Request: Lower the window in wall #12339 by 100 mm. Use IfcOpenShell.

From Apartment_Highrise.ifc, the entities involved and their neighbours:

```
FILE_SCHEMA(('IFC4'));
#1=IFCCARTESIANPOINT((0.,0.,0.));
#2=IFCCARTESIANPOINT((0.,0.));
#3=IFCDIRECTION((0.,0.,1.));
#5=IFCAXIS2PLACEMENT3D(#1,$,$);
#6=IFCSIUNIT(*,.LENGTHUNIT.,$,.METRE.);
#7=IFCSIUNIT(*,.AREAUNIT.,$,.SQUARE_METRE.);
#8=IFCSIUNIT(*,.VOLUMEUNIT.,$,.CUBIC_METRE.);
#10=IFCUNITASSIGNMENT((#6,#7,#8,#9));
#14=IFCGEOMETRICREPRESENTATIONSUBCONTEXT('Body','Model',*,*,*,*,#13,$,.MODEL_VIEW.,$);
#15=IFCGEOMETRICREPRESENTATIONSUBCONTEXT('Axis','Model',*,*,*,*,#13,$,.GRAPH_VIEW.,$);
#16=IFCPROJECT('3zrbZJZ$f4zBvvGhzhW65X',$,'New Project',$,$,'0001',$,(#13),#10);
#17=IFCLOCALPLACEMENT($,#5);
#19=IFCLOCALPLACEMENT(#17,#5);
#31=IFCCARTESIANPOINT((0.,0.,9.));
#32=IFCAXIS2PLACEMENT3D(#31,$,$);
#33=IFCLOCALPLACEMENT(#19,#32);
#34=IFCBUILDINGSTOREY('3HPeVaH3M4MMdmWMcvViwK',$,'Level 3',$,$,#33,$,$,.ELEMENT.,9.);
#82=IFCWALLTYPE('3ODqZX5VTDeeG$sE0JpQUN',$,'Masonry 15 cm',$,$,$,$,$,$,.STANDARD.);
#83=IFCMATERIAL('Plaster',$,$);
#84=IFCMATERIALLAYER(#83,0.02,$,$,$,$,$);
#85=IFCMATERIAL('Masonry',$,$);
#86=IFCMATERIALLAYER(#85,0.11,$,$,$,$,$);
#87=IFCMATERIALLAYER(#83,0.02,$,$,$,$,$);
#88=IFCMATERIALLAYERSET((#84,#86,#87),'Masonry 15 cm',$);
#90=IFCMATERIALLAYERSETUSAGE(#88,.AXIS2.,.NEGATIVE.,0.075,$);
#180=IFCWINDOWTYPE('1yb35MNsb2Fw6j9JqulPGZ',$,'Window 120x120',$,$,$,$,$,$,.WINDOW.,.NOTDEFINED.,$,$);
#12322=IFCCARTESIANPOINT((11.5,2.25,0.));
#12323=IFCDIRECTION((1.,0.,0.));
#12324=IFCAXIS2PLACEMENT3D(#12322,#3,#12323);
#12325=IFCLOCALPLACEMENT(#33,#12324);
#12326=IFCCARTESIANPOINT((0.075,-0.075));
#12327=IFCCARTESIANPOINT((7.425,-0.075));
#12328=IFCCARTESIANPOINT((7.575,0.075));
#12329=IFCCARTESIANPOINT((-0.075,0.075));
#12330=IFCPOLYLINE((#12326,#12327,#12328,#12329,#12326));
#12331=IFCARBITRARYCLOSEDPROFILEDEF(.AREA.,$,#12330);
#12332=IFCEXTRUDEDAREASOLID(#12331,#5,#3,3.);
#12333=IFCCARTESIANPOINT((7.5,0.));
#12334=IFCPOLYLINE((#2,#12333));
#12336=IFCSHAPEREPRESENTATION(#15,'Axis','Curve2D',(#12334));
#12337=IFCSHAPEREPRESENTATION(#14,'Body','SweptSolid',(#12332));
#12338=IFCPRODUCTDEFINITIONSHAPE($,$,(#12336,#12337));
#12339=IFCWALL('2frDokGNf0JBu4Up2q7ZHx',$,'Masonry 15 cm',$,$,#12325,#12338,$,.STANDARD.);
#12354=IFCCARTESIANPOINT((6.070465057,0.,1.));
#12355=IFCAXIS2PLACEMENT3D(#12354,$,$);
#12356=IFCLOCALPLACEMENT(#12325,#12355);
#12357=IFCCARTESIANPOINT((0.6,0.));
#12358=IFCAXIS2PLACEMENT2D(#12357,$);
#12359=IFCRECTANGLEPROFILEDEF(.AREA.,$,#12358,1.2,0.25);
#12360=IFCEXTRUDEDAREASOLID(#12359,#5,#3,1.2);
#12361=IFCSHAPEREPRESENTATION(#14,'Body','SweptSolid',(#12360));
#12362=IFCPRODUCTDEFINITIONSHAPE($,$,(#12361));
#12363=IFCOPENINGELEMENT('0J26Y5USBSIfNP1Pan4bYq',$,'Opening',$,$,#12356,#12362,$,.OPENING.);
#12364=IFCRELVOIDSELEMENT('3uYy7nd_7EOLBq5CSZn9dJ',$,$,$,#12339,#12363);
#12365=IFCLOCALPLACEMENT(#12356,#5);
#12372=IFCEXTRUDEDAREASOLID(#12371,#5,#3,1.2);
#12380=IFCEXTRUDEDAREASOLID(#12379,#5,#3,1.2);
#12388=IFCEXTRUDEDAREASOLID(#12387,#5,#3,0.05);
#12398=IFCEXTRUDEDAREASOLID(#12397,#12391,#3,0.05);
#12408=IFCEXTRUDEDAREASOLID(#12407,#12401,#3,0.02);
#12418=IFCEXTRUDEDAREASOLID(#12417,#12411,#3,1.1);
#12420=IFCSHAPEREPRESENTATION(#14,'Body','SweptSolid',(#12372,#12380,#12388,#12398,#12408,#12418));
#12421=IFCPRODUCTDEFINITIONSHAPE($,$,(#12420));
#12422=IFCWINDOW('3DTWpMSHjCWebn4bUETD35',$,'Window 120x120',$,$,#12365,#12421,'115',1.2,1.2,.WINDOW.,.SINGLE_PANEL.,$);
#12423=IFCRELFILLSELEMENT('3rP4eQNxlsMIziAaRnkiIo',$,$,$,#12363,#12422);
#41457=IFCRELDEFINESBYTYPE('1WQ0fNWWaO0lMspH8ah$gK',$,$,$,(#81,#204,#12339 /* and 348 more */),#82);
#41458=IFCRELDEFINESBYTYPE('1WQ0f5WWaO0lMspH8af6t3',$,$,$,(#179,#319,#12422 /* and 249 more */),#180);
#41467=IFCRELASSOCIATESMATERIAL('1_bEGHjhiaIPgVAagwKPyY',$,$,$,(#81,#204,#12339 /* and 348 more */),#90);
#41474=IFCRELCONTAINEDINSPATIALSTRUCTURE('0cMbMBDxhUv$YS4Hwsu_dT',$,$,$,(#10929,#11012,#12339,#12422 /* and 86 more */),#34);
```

```python
import numpy as np
import ifcopenshell
import ifcopenshell.api.geometry
import ifcopenshell.util.placement
import ifcopenshell.util.unit

model = ifcopenshell.open("Apartment_Highrise.ifc")
unit_scale = ifcopenshell.util.unit.calculate_unit_scale(model)

window = model.by_id(12422)
opening = window.FillsVoids[0].RelatingOpeningElement
dz = -0.1 / unit_scale

shift = np.array([0.0, 0.0, dz])
# The window is placed relative to its opening, so it follows when the opening moves.
matrix = ifcopenshell.util.placement.get_local_placement(opening.ObjectPlacement)
matrix[:3, 3] += shift
ifcopenshell.api.geometry.edit_object_placement(
    model, product=opening, matrix=matrix, is_si=False, should_transform_children=True
)

print(f"moved by {dz * unit_scale:+.3f} m")

model.write("Apartment_Highrise_rev.ifc")
```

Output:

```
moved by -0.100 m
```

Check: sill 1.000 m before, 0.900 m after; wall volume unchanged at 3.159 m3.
